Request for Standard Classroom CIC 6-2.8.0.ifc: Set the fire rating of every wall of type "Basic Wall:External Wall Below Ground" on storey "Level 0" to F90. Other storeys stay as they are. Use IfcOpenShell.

First a look at what the model holds.

```python
import ifcopenshell
import ifcopenshell.util.element

model = ifcopenshell.open("Standard Classroom CIC 6-2.8.0.ifc")
print(model.schema)
storey = next(s for s in model.by_type("IfcBuildingStorey") if s.Name == "Level 0")
walls = [e for e in ifcopenshell.util.element.get_decomposition(storey) if e.is_a("IfcWall")]
seen = {}
for e in walls:
    element_type = ifcopenshell.util.element.get_type(e)
    key = (element_type.Name if element_type != e and element_type else None, ifcopenshell.util.element.get_pset(e, "Pset_WallCommon", "FireRating"))
    seen[key] = seen.get(key, 0) + 1
for (name, value), count in sorted(seen.items(), key=str):
    print(count, "x", name, "|", value)
```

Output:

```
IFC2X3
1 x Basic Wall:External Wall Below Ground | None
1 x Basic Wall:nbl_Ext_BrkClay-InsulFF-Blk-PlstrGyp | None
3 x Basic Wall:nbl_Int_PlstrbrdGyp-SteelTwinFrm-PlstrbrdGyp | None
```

```python
import ifcopenshell
import ifcopenshell.api.pset
import ifcopenshell.util.element

model = ifcopenshell.open("Standard Classroom CIC 6-2.8.0.ifc")

storey = next(s for s in model.by_type("IfcBuildingStorey") if s.Name == "Level 0")
walls = [e for e in ifcopenshell.util.element.get_decomposition(storey) if e.is_a("IfcWall")]

count = 0
for e in walls:
    element_type = ifcopenshell.util.element.get_type(e)
    if element_type in (None, e) or element_type.Name != "Basic Wall:External Wall Below Ground":
        continue
    # add_pset returns the element's existing set when there is one.
    pset = ifcopenshell.api.pset.add_pset(model, product=e, name="Pset_WallCommon")
    ifcopenshell.api.pset.edit_pset(model, pset=pset, properties={"FireRating": "F90"})
    count += 1

print(count, "walls updated")

model.write("Standard Classroom CIC 6-2.8.0_updated.ifc")
```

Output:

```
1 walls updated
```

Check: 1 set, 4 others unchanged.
